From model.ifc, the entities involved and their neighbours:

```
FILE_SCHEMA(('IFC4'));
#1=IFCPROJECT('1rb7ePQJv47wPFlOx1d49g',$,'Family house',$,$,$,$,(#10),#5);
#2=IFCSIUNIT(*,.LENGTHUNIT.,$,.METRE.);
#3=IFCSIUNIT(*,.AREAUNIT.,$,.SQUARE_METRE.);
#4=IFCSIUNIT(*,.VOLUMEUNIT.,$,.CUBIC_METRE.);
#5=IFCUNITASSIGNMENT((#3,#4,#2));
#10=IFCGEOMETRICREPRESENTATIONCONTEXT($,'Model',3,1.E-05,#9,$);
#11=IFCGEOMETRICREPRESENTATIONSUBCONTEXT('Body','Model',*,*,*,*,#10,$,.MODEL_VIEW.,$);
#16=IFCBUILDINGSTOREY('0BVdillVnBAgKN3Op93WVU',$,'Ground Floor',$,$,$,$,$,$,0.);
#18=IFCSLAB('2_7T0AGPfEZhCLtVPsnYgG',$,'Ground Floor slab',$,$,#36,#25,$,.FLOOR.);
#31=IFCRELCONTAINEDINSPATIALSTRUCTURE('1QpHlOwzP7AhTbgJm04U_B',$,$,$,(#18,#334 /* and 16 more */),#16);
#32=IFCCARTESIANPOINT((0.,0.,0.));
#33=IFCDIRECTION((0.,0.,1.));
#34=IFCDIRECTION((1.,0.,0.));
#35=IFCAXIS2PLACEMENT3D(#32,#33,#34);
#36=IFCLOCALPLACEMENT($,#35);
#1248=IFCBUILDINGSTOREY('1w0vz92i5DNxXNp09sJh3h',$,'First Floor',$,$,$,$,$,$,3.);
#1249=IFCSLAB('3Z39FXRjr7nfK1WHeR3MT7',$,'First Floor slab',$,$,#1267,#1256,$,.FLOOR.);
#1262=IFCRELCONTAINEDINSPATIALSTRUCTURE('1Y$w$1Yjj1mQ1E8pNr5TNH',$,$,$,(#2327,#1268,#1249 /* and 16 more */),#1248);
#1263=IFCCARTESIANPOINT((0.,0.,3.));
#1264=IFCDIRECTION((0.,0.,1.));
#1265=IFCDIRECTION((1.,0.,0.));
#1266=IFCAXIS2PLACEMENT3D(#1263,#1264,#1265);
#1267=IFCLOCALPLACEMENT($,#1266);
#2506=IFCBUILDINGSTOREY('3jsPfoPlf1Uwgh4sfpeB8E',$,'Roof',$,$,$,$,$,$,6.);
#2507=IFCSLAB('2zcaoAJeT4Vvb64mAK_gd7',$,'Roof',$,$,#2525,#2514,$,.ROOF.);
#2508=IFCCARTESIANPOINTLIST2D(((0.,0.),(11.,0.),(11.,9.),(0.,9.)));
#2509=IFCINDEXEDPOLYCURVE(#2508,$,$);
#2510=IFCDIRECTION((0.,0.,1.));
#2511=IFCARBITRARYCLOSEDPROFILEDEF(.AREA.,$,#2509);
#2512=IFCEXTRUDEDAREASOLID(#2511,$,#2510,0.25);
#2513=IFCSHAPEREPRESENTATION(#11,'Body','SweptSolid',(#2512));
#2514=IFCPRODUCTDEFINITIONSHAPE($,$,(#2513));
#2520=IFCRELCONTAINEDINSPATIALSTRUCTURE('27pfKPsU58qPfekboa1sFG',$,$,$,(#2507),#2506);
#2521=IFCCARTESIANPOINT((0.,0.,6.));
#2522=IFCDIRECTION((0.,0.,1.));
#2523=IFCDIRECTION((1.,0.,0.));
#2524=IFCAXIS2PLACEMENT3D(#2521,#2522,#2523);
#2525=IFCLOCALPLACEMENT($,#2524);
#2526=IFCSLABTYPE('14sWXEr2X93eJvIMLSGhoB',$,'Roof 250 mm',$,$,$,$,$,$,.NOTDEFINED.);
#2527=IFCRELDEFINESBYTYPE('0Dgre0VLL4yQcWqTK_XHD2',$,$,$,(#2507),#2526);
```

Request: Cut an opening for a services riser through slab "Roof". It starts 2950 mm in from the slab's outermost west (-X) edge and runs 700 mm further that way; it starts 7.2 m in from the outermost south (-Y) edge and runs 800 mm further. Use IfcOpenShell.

```python
import numpy as np
import ifcopenshell
import ifcopenshell.api.feature
import ifcopenshell.api.geometry
import ifcopenshell.api.root
import ifcopenshell.geom
import ifcopenshell.util.placement
import ifcopenshell.util.representation
import ifcopenshell.util.shape
import ifcopenshell.util.unit

model = ifcopenshell.open("model.ifc")
unit_scale = ifcopenshell.util.unit.calculate_unit_scale(model)
settings = ifcopenshell.geom.settings()


def volume(element):
    """Net volume in cubic metres, openings subtracted."""
    shape = ifcopenshell.geom.create_shape(settings, element)
    return ifcopenshell.util.shape.get_volume(shape.geometry)


slab = model.by_guid("2zcaoAJeT4Vvb64mAK_gd7")
before = volume(slab)

# Extent in the slab's own axes, in metres. The edges named are its -X and -Y sides.
slab_shape = ifcopenshell.geom.create_shape(settings, slab)
vertices = ifcopenshell.util.shape.get_vertices(slab_shape.geometry)
x_min, y_min, bottom = vertices.min(axis=0)
top = vertices[:, 2].max()

opening = ifcopenshell.api.root.create_entity(model, ifc_class="IfcOpeningElement", name="Services riser opening", predefined_type="OPENING")
context = ifcopenshell.util.representation.get_context(model, "Model", "Body", "MODEL_VIEW")
width, depth = 0.7, 0.8
outline = [(0.0, 0.0), (width, 0.0), (width, depth), (0.0, depth), (0.0, 0.0)]
# Overshoot both faces by 50 mm so the cut is clean.
shape = ifcopenshell.api.geometry.add_slab_representation(
    model, context=context, depth=top - bottom + 0.1, polyline=outline
)
ifcopenshell.api.geometry.assign_representation(model, product=opening, representation=shape)

matrix = ifcopenshell.util.placement.get_local_placement(slab.ObjectPlacement)
matrix[:, 3] = matrix @ np.append(np.array([x_min + 2.95, y_min + 7.2, bottom - 0.05]) / unit_scale, 1.0)
ifcopenshell.api.geometry.edit_object_placement(model, product=opening, matrix=matrix, is_si=False)
ifcopenshell.api.feature.add_feature(model, feature=opening, element=slab)

after = volume(slab)

print(f"slab volume {before:.3f} -> {after:.3f} m3")

model.write("model-out.ifc")
```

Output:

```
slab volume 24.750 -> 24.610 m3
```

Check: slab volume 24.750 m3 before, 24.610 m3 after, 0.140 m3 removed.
